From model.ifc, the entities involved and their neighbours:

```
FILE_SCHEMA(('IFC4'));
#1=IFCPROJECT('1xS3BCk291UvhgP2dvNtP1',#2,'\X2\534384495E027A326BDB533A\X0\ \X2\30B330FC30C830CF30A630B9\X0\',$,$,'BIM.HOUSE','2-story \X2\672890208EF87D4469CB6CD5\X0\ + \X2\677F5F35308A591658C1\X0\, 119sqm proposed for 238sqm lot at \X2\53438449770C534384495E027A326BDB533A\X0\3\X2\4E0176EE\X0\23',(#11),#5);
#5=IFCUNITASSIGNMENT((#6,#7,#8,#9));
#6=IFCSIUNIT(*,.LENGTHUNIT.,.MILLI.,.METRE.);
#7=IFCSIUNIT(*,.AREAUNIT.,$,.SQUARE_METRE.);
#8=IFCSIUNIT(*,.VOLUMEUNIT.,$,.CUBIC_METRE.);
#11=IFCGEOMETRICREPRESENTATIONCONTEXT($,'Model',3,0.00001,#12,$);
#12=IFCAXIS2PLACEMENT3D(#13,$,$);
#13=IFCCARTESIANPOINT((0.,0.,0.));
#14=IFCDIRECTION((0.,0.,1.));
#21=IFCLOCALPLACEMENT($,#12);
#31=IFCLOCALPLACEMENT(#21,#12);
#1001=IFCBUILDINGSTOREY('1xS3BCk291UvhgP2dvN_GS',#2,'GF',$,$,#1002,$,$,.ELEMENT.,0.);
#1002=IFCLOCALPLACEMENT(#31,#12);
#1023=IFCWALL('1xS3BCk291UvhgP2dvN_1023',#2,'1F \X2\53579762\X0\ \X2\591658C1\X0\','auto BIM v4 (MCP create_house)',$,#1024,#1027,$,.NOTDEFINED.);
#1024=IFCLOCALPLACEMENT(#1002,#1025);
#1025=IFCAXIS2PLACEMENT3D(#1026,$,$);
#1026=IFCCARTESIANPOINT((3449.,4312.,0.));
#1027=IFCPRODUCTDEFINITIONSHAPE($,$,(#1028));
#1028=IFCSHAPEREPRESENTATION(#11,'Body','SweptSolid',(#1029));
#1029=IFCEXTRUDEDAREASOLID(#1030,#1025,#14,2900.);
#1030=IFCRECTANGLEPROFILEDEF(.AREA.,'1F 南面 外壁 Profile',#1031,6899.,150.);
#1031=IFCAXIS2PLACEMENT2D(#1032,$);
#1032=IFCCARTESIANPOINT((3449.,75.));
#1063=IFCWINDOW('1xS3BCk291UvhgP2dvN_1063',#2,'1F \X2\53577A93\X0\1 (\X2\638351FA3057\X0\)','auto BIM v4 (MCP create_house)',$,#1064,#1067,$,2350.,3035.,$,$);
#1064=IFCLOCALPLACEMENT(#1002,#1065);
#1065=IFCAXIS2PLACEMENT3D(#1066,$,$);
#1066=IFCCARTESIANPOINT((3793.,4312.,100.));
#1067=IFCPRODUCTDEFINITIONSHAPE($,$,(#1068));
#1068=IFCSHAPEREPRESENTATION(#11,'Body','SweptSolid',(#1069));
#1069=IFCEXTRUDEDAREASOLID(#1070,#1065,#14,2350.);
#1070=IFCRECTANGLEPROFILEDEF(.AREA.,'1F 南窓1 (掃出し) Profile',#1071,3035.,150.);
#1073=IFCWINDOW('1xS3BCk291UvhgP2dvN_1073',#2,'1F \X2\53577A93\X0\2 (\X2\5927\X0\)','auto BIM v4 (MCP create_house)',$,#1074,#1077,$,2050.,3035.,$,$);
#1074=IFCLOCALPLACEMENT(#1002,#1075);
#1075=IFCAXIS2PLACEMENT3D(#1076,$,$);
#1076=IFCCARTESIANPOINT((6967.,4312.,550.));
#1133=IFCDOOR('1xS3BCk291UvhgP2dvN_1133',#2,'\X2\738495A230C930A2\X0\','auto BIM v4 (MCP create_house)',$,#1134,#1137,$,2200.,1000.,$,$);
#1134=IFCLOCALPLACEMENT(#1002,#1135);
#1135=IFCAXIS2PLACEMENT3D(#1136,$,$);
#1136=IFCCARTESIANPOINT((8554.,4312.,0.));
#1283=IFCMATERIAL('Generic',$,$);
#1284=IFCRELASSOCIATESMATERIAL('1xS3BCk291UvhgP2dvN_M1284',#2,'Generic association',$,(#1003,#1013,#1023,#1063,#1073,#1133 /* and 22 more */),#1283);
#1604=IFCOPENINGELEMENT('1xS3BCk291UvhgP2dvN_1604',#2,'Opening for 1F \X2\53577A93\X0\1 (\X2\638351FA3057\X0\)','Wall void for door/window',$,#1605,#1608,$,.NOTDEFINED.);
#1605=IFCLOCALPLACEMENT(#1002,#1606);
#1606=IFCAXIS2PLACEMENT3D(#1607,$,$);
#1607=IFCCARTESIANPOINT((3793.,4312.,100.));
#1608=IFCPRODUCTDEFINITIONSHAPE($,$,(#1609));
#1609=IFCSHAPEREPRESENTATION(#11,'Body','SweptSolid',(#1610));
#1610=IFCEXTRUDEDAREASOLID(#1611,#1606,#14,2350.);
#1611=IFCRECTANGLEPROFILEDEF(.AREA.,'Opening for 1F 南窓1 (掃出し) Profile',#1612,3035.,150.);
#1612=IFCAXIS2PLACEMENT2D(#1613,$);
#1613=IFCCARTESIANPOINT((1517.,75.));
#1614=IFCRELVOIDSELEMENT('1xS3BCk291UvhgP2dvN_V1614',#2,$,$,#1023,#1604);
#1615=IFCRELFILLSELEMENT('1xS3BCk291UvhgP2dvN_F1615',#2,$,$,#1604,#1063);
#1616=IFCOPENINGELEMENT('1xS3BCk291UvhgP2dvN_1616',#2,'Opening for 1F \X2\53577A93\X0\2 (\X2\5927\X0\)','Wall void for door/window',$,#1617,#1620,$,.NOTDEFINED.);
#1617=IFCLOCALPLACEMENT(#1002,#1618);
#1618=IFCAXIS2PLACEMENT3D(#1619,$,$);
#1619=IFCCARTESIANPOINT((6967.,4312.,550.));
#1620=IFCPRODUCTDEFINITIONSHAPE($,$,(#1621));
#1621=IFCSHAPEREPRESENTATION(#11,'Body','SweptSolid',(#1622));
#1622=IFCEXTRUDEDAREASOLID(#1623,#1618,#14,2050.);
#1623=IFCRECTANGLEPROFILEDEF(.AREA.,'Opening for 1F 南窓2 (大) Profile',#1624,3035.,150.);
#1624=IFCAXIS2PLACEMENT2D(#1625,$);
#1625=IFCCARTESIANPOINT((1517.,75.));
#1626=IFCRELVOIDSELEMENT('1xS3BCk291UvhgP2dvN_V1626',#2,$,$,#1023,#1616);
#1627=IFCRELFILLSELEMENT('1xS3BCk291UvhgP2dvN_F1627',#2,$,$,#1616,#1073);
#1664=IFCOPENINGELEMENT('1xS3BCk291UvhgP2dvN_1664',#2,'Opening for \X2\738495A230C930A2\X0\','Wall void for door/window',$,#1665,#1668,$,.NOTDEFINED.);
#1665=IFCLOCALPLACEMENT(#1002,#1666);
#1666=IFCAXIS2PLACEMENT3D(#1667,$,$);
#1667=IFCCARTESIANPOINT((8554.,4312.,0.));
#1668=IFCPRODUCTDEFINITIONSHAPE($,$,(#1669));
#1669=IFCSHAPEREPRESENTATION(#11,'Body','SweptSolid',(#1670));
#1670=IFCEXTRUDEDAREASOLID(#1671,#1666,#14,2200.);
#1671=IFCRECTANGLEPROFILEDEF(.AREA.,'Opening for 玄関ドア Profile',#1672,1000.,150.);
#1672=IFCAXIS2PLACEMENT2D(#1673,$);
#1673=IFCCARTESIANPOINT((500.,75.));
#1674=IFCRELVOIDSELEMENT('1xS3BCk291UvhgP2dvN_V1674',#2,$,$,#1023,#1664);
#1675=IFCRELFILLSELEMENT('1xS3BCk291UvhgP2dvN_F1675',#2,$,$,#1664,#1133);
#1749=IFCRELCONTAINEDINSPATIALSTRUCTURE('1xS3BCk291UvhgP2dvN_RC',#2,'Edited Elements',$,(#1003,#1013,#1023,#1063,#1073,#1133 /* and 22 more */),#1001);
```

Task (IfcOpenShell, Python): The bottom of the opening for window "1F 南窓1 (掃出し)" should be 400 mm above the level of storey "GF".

```python
import numpy as np
import ifcopenshell
import ifcopenshell.api.geometry
import ifcopenshell.geom
import ifcopenshell.util.element
import ifcopenshell.util.placement
import ifcopenshell.util.shape
import ifcopenshell.util.unit

model = ifcopenshell.open("model.ifc")
unit_scale = ifcopenshell.util.unit.calculate_unit_scale(model)

window = model.by_guid("1xS3BCk291UvhgP2dvN_1063")
opening = window.FillsVoids[0].RelatingOpeningElement
storey = ifcopenshell.util.element.get_container(window, ifc_class="IfcBuildingStorey")
level = ifcopenshell.util.placement.get_local_placement(storey.ObjectPlacement)[2, 3]

# The opening's origin need not be at the sill, so measure its lowest point.
shape = ifcopenshell.geom.create_shape(ifcopenshell.geom.settings(), opening)
bottom = ifcopenshell.util.shape.get_shape_bottom_elevation(shape, shape.geometry) / unit_scale
dz = level + 400.0 - bottom

shift = np.array([0.0, 0.0, dz])
# The window is not placed relative to its opening, so move both.
for product in (opening, window):
    matrix = ifcopenshell.util.placement.get_local_placement(product.ObjectPlacement)
    matrix[:3, 3] += shift
    ifcopenshell.api.geometry.edit_object_placement(model, product=product, matrix=matrix, is_si=False)

print(f"moved by {dz * unit_scale:+.3f} m")

model.write("model_v2.ifc")
```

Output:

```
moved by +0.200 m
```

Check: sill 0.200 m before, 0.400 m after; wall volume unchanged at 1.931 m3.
